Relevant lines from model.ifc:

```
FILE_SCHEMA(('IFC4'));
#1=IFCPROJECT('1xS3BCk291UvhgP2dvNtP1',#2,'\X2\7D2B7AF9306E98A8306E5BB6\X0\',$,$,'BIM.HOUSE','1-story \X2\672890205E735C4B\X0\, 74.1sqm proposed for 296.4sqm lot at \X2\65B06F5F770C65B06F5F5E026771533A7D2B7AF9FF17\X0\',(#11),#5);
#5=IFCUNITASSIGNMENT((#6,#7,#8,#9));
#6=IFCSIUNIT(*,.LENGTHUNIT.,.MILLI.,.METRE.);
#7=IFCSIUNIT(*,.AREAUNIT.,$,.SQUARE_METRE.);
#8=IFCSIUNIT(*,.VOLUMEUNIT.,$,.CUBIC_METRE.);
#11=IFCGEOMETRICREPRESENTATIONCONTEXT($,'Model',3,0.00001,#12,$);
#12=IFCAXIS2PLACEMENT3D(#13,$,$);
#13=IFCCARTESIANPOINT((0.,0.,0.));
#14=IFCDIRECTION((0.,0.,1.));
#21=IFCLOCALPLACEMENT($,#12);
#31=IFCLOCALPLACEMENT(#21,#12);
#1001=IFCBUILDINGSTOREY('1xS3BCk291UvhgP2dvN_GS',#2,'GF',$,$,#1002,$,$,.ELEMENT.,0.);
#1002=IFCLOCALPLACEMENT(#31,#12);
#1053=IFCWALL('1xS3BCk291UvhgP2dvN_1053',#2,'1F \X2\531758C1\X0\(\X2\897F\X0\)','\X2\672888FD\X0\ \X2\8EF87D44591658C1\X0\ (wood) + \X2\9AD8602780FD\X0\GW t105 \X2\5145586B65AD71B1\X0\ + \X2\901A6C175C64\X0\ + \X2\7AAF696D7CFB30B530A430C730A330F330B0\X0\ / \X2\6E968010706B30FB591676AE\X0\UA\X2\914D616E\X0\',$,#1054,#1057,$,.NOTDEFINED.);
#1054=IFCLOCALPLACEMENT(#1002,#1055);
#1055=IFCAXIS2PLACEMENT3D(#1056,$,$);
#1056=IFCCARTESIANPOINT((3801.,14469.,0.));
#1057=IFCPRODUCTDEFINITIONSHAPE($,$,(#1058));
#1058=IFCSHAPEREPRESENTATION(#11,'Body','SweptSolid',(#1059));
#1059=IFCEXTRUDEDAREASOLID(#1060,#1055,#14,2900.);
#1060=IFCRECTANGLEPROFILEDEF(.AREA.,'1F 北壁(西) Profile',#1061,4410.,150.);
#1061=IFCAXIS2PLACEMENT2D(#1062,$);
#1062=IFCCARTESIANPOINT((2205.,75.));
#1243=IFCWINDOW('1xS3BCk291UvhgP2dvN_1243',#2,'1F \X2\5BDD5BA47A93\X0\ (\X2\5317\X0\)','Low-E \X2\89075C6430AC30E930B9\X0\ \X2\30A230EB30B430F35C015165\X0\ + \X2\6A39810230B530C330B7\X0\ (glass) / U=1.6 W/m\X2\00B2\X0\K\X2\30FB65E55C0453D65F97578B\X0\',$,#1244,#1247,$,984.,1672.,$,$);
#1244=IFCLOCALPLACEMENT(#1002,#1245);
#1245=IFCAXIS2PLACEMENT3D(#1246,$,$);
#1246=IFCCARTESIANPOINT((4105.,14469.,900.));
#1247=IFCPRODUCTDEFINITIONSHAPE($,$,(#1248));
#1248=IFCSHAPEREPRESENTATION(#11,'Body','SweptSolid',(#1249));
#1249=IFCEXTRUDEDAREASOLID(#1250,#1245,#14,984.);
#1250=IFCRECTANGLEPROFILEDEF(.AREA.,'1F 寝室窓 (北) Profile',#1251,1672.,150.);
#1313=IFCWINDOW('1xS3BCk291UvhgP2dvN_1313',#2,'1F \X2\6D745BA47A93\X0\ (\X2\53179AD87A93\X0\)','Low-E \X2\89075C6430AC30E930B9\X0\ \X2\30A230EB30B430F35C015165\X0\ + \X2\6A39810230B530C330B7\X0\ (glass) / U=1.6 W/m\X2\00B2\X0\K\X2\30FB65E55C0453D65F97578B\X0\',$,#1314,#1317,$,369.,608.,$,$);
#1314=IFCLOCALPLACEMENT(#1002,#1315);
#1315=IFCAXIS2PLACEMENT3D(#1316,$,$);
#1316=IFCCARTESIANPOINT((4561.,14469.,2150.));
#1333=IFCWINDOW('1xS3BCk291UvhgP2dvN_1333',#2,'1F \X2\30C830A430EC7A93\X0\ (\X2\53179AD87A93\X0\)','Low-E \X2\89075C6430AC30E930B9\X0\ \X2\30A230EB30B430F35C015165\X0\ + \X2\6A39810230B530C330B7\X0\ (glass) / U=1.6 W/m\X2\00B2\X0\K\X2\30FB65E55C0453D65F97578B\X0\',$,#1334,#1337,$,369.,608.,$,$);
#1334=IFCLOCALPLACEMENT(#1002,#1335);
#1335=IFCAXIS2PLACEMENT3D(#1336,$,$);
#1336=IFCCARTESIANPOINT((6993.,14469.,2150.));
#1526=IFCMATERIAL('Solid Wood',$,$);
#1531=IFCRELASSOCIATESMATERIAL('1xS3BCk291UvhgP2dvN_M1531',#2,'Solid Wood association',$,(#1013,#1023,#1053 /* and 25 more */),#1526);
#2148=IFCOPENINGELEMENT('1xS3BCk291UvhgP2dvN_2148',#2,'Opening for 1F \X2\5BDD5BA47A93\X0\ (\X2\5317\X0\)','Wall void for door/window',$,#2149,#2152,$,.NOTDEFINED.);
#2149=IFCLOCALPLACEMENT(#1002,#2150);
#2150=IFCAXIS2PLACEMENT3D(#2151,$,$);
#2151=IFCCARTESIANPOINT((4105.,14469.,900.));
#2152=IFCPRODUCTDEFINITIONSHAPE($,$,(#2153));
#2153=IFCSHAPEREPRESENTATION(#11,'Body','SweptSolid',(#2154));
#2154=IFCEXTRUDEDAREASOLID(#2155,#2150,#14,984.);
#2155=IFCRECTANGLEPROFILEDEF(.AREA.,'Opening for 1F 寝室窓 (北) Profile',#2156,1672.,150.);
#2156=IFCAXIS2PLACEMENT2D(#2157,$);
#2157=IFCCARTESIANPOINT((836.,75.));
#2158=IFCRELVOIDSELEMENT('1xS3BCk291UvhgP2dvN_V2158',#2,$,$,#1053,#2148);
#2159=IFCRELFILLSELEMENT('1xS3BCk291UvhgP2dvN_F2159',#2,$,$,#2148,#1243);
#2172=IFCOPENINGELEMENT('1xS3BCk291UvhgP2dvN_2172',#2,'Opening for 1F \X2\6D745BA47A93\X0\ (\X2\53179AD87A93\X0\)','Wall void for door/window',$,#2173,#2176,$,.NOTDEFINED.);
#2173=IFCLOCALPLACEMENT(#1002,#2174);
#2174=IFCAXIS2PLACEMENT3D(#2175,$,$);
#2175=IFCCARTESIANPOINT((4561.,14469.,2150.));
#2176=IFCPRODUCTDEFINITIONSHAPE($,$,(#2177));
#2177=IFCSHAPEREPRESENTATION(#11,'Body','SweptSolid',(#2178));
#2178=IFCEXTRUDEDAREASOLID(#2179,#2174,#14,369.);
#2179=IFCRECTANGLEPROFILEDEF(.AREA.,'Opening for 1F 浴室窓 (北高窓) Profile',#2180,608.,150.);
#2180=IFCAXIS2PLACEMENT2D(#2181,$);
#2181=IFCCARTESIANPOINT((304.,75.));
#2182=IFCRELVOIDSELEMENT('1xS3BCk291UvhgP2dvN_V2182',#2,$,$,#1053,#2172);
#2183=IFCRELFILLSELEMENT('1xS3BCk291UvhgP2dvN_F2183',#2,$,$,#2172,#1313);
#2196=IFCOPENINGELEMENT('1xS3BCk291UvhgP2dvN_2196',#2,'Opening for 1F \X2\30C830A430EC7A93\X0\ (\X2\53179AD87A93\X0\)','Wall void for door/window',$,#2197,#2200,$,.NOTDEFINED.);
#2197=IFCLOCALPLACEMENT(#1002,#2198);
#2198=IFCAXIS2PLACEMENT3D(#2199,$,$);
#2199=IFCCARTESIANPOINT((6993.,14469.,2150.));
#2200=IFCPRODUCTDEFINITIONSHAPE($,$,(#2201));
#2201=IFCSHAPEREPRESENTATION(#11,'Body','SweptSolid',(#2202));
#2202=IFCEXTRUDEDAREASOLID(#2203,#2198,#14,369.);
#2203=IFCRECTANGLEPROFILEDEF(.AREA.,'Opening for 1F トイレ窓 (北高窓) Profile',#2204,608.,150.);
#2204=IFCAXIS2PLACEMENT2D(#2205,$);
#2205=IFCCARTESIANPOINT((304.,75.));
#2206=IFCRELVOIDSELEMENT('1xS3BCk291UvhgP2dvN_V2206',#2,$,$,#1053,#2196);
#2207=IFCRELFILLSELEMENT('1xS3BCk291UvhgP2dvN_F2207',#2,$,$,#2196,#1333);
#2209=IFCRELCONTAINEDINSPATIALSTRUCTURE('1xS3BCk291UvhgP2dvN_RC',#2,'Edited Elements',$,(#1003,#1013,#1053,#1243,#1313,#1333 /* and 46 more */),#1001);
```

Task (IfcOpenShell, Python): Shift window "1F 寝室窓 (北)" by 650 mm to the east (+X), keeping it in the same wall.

```python
import ifcopenshell
import ifcopenshell.api.geometry
import ifcopenshell.util.placement
import ifcopenshell.util.unit

model = ifcopenshell.open("model.ifc")
unit_scale = ifcopenshell.util.unit.calculate_unit_scale(model)

window = model.by_id(1243)
opening = window.FillsVoids[0].RelatingOpeningElement
wall = opening.VoidsElements[0].RelatingBuildingElement

wall_matrix = ifcopenshell.util.placement.get_local_placement(wall.ObjectPlacement)
shift = wall_matrix[:3, 0] * 0.65 / unit_scale
before = ifcopenshell.util.placement.get_local_placement(window.ObjectPlacement)[:3, 3].copy()

# The window is not placed relative to its opening, so move both.
for product in (opening, window):
    matrix = ifcopenshell.util.placement.get_local_placement(product.ObjectPlacement)
    matrix[:3, 3] += shift
    ifcopenshell.api.geometry.edit_object_placement(model, product=product, matrix=matrix, is_si=False)

after = ifcopenshell.util.placement.get_local_placement(window.ObjectPlacement)[:3, 3]
print("window moved by", (after - before).round(3) + 0.0)

model.write("model_rev.ifc")
```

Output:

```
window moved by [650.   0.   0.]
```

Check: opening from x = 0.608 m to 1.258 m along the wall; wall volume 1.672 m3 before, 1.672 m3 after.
